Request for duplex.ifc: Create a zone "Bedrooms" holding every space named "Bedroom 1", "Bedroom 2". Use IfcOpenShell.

First a look at what the model holds.

```python
import ifcopenshell

model = ifcopenshell.open("duplex.ifc")
print(model.schema)
seen = {}
for space in model.by_type("IfcSpace"):
    seen[space.LongName] = seen.get(space.LongName, 0) + 1
for name, count in sorted(seen.items(), key=str):
    print(count, "x", name)
print("zones:", [z.Name for z in model.by_type("IfcZone")][:20])
```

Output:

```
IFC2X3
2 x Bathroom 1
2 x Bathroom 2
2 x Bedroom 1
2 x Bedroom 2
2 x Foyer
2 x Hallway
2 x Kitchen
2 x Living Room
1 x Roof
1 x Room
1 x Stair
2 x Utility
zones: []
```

```python
import ifcopenshell
import ifcopenshell.api.group
import ifcopenshell.api.root

model = ifcopenshell.open("duplex.ifc")

names = {"Bedroom 1", "Bedroom 2"}
spaces = [s for s in model.by_type("IfcSpace") if s.LongName in names]

zone = ifcopenshell.api.root.create_entity(model, ifc_class="IfcZone", name="Bedrooms")
ifcopenshell.api.group.assign_group(model, products=spaces, group=zone)
print(len(spaces), "spaces in", zone.Name)

model.write("duplex_v2.ifc")
```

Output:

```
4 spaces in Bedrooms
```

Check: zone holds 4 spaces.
